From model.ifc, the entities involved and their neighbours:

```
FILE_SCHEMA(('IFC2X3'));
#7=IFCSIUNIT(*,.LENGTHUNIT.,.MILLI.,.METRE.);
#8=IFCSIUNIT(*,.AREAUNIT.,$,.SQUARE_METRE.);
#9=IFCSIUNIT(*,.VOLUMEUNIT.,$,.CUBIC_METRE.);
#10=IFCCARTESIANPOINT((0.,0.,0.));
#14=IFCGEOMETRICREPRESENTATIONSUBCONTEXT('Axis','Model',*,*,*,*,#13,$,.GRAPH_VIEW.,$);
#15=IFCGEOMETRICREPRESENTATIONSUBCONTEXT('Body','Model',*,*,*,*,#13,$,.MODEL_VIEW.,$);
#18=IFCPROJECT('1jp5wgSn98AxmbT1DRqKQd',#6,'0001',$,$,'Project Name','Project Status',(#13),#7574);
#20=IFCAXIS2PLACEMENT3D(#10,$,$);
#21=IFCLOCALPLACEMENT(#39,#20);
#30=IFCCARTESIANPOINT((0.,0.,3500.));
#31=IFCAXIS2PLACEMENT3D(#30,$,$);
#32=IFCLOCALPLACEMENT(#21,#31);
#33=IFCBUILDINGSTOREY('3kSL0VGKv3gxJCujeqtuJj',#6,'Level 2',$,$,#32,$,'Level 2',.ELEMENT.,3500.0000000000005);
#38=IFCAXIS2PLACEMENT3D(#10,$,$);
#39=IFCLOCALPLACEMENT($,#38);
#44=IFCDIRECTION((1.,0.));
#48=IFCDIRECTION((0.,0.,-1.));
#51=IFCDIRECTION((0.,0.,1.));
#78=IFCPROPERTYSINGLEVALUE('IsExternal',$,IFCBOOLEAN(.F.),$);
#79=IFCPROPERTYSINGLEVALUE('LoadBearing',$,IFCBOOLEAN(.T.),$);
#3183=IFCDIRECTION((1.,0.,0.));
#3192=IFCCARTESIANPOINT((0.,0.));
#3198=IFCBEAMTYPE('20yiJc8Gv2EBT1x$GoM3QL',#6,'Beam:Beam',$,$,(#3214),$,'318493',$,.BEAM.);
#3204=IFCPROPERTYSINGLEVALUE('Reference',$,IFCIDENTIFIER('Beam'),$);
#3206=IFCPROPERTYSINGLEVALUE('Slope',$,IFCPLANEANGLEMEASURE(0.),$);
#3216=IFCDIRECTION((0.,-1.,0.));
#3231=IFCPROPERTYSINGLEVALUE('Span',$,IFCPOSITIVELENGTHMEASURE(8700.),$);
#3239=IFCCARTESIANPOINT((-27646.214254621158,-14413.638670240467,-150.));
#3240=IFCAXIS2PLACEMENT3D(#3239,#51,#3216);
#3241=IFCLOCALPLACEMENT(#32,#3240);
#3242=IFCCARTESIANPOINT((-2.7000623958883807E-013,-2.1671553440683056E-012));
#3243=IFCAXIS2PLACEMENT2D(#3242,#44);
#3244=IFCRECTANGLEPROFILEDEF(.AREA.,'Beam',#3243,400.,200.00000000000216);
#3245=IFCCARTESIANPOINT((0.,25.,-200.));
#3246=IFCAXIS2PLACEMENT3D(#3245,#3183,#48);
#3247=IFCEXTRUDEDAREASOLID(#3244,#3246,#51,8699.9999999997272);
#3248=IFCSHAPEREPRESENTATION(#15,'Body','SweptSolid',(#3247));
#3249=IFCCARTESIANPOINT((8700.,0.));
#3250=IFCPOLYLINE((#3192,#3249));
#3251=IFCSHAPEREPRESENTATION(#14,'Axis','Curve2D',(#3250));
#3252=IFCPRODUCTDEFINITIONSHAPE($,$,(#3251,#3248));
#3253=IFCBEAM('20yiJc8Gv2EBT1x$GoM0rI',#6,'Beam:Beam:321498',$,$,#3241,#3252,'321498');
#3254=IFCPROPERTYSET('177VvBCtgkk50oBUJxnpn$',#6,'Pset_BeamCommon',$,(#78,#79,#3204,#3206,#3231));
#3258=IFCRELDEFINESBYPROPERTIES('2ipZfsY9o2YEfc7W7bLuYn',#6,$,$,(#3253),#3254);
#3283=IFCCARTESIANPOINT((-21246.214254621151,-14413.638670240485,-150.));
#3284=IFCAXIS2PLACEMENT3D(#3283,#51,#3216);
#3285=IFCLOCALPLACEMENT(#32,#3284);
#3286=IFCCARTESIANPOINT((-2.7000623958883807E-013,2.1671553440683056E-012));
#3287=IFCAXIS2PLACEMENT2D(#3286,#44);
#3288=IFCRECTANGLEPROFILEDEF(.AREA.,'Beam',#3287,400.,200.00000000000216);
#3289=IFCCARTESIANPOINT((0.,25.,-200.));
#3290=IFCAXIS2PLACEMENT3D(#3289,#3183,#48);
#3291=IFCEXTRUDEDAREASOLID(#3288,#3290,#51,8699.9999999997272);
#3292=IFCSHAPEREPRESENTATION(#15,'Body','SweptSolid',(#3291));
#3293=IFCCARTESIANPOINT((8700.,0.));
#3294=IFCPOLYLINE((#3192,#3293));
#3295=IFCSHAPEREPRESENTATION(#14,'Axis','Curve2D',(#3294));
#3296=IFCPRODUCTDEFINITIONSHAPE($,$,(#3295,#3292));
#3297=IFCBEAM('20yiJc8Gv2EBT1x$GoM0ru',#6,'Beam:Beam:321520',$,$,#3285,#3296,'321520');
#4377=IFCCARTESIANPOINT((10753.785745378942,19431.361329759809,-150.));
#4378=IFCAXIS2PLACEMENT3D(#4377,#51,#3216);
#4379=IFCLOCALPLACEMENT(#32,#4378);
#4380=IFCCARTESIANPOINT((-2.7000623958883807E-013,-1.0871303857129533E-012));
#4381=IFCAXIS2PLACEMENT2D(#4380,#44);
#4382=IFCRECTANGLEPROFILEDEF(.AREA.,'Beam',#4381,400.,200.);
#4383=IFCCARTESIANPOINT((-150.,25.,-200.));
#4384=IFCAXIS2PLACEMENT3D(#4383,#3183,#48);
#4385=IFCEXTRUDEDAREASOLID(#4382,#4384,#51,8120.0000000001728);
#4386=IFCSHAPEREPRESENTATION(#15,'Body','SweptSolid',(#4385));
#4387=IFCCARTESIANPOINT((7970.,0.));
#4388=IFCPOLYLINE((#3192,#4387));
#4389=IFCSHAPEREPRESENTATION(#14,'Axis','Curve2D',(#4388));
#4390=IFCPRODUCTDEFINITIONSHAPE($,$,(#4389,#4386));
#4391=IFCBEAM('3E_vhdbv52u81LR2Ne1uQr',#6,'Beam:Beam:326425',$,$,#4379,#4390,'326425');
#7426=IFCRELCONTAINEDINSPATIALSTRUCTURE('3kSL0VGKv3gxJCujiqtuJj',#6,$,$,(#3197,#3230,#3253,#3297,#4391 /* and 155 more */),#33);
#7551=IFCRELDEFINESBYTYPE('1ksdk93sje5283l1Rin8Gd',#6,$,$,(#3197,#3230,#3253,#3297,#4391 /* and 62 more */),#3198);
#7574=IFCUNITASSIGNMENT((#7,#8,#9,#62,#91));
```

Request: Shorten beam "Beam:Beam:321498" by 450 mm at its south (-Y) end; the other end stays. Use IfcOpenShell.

```python
import numpy as np
import ifcopenshell
import ifcopenshell.api.pset
import ifcopenshell.util.element
import ifcopenshell.util.representation
import ifcopenshell.util.unit

model = ifcopenshell.open("model.ifc")
unit_scale = ifcopenshell.util.unit.calculate_unit_scale(model)

member = model.by_guid("20yiJc8Gv2EBT1x$GoM0rI")
change = -0.45 / unit_scale

# The extrusion runs towards the end named, so only its depth changes.
body = ifcopenshell.util.representation.get_representation(member, "Model", "Body")
solid = body.Items[0]
old_length = solid.Depth
solid.Depth += change

# Move the axis end point with it.
axis = next(r for r in member.Representation.Representations if r.RepresentationIdentifier == "Axis").Items[0]
start, end = (np.array(p.Coordinates) for p in axis.Points)
end = end + (end - start) / np.linalg.norm(end - start) * change
point = model.createIfcCartesianPoint(end.tolist())
axis.Points = [axis.Points[0], point]

# Update the stored length and volume.
pset = model.by_id(ifcopenshell.util.element.get_pset(member, "Pset_BeamCommon", should_inherit=False)["id"])
ifcopenshell.api.pset.edit_pset(model, pset=pset, properties={
    "Span": model.create_entity("IfcPositiveLengthMeasure", solid.Depth),
})

print(f"length {old_length:g} -> {solid.Depth:g}")

model.write("model-out.ifc")
```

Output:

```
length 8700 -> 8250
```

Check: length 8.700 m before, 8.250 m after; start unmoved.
